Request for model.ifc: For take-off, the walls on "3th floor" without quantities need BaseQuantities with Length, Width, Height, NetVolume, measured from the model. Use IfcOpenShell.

First a look at what the model holds.

```python
import ifcopenshell
import ifcopenshell.util.element
import ifcopenshell.util.unit

model = ifcopenshell.open("model.ifc")
print(model.schema)
for unit_type in ("LENGTHUNIT", "AREAUNIT", "VOLUMEUNIT"):
    print(unit_type, ifcopenshell.util.unit.calculate_unit_scale(model, unit_type))
storey = next(s for s in model.by_type("IfcBuildingStorey") if s.Name == "3th floor")
walls = [e for e in ifcopenshell.util.element.get_decomposition(storey) if e.is_a("IfcWall")]
for e in sorted(walls, key=lambda e: e.id()):
    print(e.id(), e.is_a(), e.Name, list(ifcopenshell.util.element.get_psets(e, qtos_only=True)), sep=" | ")
```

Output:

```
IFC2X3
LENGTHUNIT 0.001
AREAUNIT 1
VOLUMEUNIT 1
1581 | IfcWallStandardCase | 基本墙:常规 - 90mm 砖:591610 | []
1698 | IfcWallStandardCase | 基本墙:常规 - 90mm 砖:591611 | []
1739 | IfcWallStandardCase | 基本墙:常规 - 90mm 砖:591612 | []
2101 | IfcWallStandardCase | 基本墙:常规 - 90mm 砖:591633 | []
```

```python
import ifcopenshell
import ifcopenshell.api.pset
import ifcopenshell.geom
import ifcopenshell.util.element
import ifcopenshell.util.shape
import ifcopenshell.util.unit

model = ifcopenshell.open("model.ifc")
unit_scale = ifcopenshell.util.unit.calculate_unit_scale(model)
volume_scale = ifcopenshell.util.unit.calculate_unit_scale(model, "VOLUMEUNIT")
settings = ifcopenshell.geom.settings()

storey = next(s for s in model.by_type("IfcBuildingStorey") if s.Name == "3th floor")
walls = [e for e in ifcopenshell.util.element.get_decomposition(storey) if e.is_a("IfcWall")]

for e in sorted(walls, key=lambda e: e.id()):
    if ifcopenshell.util.element.get_psets(e, qtos_only=True, should_inherit=False):
        continue
    # Geometry comes back in metres, in the element's own axes.
    shape = ifcopenshell.geom.create_shape(settings, e)
    values = {
        "Length": ifcopenshell.util.shape.get_x(shape.geometry) / unit_scale,
        "Width": ifcopenshell.util.shape.get_y(shape.geometry) / unit_scale,
        "Height": ifcopenshell.util.shape.get_z(shape.geometry) / unit_scale,
        "NetVolume": ifcopenshell.util.shape.get_volume(shape.geometry) / volume_scale,
    }
    qto = ifcopenshell.api.pset.add_qto(model, product=e, name="BaseQuantities")
    ifcopenshell.api.pset.edit_qto(model, qto=qto, properties=values)
    print(e.id(), {k: round(v, 3) for k, v in values.items()})

model.write("model_updated.ifc")
```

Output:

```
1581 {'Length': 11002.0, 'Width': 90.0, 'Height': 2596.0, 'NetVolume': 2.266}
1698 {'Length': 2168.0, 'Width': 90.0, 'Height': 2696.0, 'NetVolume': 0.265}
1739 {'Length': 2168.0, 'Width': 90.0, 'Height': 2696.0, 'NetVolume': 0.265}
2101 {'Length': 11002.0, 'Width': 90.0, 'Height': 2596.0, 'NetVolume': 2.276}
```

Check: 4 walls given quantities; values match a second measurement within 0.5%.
